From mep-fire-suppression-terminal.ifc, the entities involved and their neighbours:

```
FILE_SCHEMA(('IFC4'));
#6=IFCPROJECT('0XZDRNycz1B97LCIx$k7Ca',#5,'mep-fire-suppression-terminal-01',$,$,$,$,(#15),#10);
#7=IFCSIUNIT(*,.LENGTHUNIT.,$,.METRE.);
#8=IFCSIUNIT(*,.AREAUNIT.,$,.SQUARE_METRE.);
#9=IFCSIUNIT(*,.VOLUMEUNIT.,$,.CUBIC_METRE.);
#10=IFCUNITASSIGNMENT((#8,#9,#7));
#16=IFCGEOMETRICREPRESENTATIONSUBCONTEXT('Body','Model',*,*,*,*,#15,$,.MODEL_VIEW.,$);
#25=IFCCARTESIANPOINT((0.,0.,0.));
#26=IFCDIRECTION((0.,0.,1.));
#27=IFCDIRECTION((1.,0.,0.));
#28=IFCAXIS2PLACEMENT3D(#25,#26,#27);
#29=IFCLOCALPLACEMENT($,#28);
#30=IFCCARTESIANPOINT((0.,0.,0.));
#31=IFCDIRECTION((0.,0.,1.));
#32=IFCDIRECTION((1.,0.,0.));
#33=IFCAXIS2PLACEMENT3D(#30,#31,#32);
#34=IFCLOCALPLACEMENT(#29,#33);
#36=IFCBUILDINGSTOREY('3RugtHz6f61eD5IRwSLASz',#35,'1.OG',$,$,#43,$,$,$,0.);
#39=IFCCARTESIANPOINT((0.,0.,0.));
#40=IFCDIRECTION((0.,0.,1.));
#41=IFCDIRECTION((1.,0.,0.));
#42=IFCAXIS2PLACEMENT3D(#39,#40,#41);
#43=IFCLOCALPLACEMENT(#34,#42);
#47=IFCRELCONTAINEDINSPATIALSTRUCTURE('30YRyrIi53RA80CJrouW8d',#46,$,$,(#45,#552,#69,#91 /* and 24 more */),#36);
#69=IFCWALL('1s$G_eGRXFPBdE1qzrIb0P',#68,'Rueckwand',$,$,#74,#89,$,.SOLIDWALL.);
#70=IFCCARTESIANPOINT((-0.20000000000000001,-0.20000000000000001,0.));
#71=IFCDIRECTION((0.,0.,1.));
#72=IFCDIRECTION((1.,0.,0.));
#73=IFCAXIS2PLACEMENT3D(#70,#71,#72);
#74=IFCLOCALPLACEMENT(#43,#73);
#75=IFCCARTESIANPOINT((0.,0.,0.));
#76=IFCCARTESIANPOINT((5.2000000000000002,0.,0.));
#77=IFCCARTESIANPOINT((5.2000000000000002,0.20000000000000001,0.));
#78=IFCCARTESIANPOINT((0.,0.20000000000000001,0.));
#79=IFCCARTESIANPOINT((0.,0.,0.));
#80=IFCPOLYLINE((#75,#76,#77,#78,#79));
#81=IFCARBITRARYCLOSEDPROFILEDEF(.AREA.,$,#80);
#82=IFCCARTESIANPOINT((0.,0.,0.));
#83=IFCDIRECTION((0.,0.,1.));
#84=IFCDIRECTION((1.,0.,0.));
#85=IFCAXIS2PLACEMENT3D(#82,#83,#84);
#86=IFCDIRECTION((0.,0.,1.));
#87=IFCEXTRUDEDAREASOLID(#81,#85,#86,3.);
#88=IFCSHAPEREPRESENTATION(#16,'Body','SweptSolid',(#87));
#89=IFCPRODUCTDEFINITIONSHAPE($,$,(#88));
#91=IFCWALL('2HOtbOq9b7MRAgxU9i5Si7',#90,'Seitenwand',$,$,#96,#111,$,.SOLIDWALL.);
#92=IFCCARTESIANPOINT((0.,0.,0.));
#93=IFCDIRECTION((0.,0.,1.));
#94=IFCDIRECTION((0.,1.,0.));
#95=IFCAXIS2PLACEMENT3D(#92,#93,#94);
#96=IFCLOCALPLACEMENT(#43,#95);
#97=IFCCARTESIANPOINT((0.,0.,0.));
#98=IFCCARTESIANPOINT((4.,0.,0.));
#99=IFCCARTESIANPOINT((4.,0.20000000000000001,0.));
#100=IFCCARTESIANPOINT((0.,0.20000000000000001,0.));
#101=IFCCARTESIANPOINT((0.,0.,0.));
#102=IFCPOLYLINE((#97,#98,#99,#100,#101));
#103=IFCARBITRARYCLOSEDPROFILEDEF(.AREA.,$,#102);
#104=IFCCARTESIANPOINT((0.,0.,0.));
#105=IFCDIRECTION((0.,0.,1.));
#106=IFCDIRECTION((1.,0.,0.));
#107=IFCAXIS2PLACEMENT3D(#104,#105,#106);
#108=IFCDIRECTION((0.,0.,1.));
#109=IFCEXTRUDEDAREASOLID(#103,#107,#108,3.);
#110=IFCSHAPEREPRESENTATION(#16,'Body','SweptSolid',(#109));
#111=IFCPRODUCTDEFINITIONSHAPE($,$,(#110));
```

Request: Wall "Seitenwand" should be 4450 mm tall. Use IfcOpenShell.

```python
import ifcopenshell
import ifcopenshell.geom
import ifcopenshell.util.representation
import ifcopenshell.util.shape
import ifcopenshell.util.unit

model = ifcopenshell.open("mep-fire-suppression-terminal.ifc")
unit_scale = ifcopenshell.util.unit.calculate_unit_scale(model)
settings = ifcopenshell.geom.settings()


def volume(element):
    """Net volume in cubic metres, openings subtracted."""
    shape = ifcopenshell.geom.create_shape(settings, element)
    return ifcopenshell.util.shape.get_volume(shape.geometry)


wall = model.by_guid("2HOtbOq9b7MRAgxU9i5Si7")
before = volume(wall)

body = ifcopenshell.util.representation.get_representation(wall, "Model", "Body")
solid = body.Items[0]
old_height = solid.Depth
solid.Depth = 4.45 / unit_scale
after = volume(wall)

print(f"height {old_height:g} -> {solid.Depth:g}, volume {before:.3f} -> {after:.3f} m3")

model.write("mep-fire-suppression-terminal_v2.ifc")
```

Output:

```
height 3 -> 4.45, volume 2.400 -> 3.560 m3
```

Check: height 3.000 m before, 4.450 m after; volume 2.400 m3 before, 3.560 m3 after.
